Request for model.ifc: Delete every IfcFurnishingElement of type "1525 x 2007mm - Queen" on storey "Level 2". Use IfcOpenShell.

First a look at what the model holds.

```python
import ifcopenshell
import ifcopenshell.util.element

model = ifcopenshell.open("model.ifc")
print(model.schema)
storey = next(s for s in model.by_type("IfcBuildingStorey") if s.Name == "Level 2")
furniture = [e for e in ifcopenshell.util.element.get_decomposition(storey) if e.is_a("IfcFurnishingElement")]
seen = {}
for e in furniture:
    element_type = ifcopenshell.util.element.get_type(e)
    name = element_type.Name if element_type not in (None, e) else None
    seen[name] = seen.get(name, 0) + 1
for name, count in sorted(seen.items(), key=str):
    print(count, "x", name)
```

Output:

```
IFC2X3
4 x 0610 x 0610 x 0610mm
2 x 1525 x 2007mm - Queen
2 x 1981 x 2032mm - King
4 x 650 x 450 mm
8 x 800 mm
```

```python
import ifcopenshell
import ifcopenshell.api.root
import ifcopenshell.util.element

model = ifcopenshell.open("model.ifc")

storey = next(s for s in model.by_type("IfcBuildingStorey") if s.Name == "Level 2")
furniture = [e for e in ifcopenshell.util.element.get_decomposition(storey) if e.is_a("IfcFurnishingElement")]
targets = [e for e in furniture if (t := ifcopenshell.util.element.get_type(e)) not in (None, e) and t.Name == "1525 x 2007mm - Queen"]

for e in targets:
    ifcopenshell.api.root.remove_product(model, product=e)
print(len(targets), "removed")

model.write("model_v2.ifc")
```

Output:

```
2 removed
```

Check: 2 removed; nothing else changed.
